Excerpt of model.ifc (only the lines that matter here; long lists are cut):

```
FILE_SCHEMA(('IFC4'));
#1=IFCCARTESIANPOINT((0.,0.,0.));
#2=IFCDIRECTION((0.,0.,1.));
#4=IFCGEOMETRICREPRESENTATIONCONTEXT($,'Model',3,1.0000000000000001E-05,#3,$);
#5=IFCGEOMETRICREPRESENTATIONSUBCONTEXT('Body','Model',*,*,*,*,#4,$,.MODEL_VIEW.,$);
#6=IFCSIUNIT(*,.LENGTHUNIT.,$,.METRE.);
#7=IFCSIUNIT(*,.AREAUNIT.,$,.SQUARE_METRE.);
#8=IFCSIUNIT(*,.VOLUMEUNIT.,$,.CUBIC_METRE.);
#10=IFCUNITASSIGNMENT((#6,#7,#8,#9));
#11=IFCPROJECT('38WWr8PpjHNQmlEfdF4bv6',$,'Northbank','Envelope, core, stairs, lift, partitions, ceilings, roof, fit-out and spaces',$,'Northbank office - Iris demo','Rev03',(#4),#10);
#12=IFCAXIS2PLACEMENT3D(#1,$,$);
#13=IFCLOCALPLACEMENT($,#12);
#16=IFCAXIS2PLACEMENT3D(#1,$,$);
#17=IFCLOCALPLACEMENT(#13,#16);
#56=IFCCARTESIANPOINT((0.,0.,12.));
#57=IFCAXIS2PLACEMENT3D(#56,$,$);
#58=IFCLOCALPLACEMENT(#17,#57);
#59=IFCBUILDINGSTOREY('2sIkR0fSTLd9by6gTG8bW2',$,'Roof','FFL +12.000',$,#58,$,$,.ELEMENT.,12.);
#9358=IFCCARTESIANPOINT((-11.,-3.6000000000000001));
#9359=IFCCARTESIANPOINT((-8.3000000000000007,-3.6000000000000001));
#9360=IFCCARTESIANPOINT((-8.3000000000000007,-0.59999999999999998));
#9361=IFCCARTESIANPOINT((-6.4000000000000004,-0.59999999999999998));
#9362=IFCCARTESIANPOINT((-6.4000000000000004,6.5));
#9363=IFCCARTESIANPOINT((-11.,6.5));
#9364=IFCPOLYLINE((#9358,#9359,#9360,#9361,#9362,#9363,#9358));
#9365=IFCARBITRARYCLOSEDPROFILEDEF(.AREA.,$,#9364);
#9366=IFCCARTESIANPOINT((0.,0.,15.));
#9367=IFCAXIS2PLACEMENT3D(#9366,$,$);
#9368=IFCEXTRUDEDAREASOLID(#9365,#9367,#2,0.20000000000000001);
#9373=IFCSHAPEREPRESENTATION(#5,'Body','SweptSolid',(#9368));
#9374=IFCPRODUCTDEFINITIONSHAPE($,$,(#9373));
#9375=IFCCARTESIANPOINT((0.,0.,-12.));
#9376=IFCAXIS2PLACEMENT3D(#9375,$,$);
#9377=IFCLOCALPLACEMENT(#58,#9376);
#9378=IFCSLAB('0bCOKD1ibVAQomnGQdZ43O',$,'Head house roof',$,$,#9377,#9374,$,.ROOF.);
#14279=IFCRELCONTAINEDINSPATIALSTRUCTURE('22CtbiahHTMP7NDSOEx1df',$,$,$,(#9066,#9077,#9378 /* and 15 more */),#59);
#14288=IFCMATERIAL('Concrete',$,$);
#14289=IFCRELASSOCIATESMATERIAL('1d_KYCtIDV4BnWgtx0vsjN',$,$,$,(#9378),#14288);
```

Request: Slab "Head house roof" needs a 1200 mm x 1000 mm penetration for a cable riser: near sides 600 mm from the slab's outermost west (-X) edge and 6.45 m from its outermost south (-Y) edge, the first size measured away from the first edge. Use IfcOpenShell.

```python
import numpy as np
import ifcopenshell
import ifcopenshell.api.feature
import ifcopenshell.api.geometry
import ifcopenshell.api.root
import ifcopenshell.geom
import ifcopenshell.util.placement
import ifcopenshell.util.representation
import ifcopenshell.util.shape
import ifcopenshell.util.unit

model = ifcopenshell.open("model.ifc")
unit_scale = ifcopenshell.util.unit.calculate_unit_scale(model)
settings = ifcopenshell.geom.settings()


def volume(element):
    """Net volume in cubic metres, openings subtracted."""
    shape = ifcopenshell.geom.create_shape(settings, element)
    return ifcopenshell.util.shape.get_volume(shape.geometry)


slab = model.by_guid("0bCOKD1ibVAQomnGQdZ43O")
before = volume(slab)

# Extent in the slab's own axes, in metres. The edges named are its -X and -Y sides.
slab_shape = ifcopenshell.geom.create_shape(settings, slab)
vertices = ifcopenshell.util.shape.get_vertices(slab_shape.geometry)
x_min, y_min, bottom = vertices.min(axis=0)
top = vertices[:, 2].max()

opening = ifcopenshell.api.root.create_entity(model, ifc_class="IfcOpeningElement", name="Cable riser opening", predefined_type="OPENING")
context = ifcopenshell.util.representation.get_context(model, "Model", "Body", "MODEL_VIEW")
width, depth = 1.2, 1
outline = [(0.0, 0.0), (width, 0.0), (width, depth), (0.0, depth), (0.0, 0.0)]
# Overshoot both faces by 50 mm so the cut is clean.
shape = ifcopenshell.api.geometry.add_slab_representation(
    model, context=context, depth=top - bottom + 0.1, polyline=outline
)
ifcopenshell.api.geometry.assign_representation(model, product=opening, representation=shape)

matrix = ifcopenshell.util.placement.get_local_placement(slab.ObjectPlacement)
matrix[:, 3] = matrix @ np.append(np.array([x_min + 0.6, y_min + 6.45, bottom - 0.05]) / unit_scale, 1.0)
ifcopenshell.api.geometry.edit_object_placement(model, product=opening, matrix=matrix, is_si=False)
ifcopenshell.api.feature.add_feature(model, feature=opening, element=slab)

after = volume(slab)

print(f"slab volume {before:.3f} -> {after:.3f} m3")

model.write("model_rev.ifc")
```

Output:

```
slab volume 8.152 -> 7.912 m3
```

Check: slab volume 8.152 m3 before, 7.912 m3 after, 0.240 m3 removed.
